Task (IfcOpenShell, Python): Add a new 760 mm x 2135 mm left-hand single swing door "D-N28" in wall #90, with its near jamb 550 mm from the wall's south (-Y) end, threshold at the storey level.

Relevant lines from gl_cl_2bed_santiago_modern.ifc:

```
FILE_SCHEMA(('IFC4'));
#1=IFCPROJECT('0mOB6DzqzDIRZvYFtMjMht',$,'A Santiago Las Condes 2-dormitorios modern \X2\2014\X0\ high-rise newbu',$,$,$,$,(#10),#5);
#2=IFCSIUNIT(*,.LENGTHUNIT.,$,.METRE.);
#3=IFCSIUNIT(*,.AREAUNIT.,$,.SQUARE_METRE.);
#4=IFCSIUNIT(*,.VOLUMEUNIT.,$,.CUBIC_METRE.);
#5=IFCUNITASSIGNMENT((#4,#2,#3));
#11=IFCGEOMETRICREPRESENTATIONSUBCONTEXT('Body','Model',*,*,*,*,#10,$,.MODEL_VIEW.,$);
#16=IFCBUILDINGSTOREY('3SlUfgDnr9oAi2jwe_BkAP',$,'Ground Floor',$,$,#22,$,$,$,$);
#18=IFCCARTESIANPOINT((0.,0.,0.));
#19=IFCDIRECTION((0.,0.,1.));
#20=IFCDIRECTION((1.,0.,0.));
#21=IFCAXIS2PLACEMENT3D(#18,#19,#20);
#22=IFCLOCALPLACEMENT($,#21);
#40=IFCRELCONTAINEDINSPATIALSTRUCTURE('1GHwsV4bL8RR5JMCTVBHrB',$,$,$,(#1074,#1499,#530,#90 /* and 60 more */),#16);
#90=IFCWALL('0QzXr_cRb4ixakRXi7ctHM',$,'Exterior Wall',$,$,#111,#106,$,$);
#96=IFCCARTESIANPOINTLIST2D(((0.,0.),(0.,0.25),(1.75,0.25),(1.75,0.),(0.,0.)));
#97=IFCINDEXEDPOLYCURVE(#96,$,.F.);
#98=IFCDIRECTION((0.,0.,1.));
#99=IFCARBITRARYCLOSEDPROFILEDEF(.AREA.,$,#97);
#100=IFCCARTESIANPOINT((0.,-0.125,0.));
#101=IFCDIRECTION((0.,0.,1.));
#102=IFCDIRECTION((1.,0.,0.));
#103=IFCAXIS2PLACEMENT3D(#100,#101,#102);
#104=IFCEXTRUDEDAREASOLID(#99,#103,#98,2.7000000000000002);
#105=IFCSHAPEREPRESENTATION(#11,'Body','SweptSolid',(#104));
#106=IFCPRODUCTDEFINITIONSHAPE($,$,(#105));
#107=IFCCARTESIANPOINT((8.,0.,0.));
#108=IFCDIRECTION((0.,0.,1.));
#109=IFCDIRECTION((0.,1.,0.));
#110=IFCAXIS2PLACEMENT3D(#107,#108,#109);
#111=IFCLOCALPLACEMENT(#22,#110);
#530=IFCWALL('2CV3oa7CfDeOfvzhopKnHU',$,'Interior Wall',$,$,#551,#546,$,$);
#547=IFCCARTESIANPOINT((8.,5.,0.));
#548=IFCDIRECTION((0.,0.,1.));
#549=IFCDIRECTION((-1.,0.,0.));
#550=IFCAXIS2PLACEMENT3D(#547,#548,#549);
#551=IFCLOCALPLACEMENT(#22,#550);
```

```python
import numpy as np
import ifcopenshell
import ifcopenshell.api.feature
import ifcopenshell.api.geometry
import ifcopenshell.api.root
import ifcopenshell.api.spatial
import ifcopenshell.geom
import ifcopenshell.util.element
import ifcopenshell.util.placement
import ifcopenshell.util.representation
import ifcopenshell.util.shape
import ifcopenshell.util.unit

model = ifcopenshell.open("gl_cl_2bed_santiago_modern.ifc")
unit_scale = ifcopenshell.util.unit.calculate_unit_scale(model)
settings = ifcopenshell.geom.settings()


def volume(element):
    """Net volume in cubic metres, openings subtracted."""
    shape = ifcopenshell.geom.create_shape(settings, element)
    return ifcopenshell.util.shape.get_volume(shape.geometry)


wall = model.by_guid("0QzXr_cRb4ixakRXi7ctHM")
storey = ifcopenshell.util.element.get_container(wall, ifc_class="IfcBuildingStorey")
context = ifcopenshell.util.representation.get_context(model, "Model", "Body", "MODEL_VIEW")
before = volume(wall)

width, height, from_end, sill = 0.76, 2.135, 0.55, 0.0  # metres

# The wall runs along its own X axis, and the end named is its -X end.
wall_shape = ifcopenshell.geom.create_shape(settings, wall)
x, y, z = ifcopenshell.util.shape.get_vertices(wall_shape.geometry).T
start = x.min() + from_end
face, thickness = float(y.min()), float(y.max() - y.min())
wall_matrix = ifcopenshell.util.placement.get_local_placement(wall.ObjectPlacement)
level = ifcopenshell.util.placement.get_local_placement(storey.ObjectPlacement)[2, 3]


def in_wall(x, y):
    """Placement at x, y metres in the wall's axes, at sill height."""
    matrix = wall_matrix.copy()
    matrix[:, 3] = wall_matrix @ np.array([x / unit_scale, y / unit_scale, 0.0, 1.0])
    matrix[2, 3] = level + sill / unit_scale
    return matrix


# Opening: a box that overshoots both wall faces by 50 mm.
opening = ifcopenshell.api.root.create_entity(model, ifc_class="IfcOpeningElement", predefined_type="OPENING")
box = ifcopenshell.api.geometry.add_wall_representation(
    model, context=context, length=width, height=height, thickness=thickness + 0.1
)
ifcopenshell.api.geometry.assign_representation(model, product=opening, representation=box)
ifcopenshell.api.geometry.edit_object_placement(model, product=opening, matrix=in_wall(start, face - 0.05), is_si=False)
ifcopenshell.api.feature.add_feature(model, feature=opening, element=wall)

door = ifcopenshell.api.root.create_entity(model, ifc_class="IfcDoor", name="D-N28", predefined_type="DOOR")
door.OverallWidth, door.OverallHeight = width / unit_scale, height / unit_scale
door.OperationType = "SINGLE_SWING_LEFT"
body = ifcopenshell.api.geometry.add_door_representation(
    model,
    context=context,
    overall_width=door.OverallWidth,
    overall_height=door.OverallHeight,
    operation_type="SINGLE_SWING_LEFT",
    lining_properties={"LiningDepth": thickness / unit_scale, "ThresholdDepth": thickness / unit_scale},
)
ifcopenshell.api.geometry.assign_representation(model, product=door, representation=body)
ifcopenshell.api.spatial.assign_container(model, products=[door], relating_structure=storey)
ifcopenshell.api.feature.add_filling(model, opening=opening, element=door)

# The lining spans the wall, so the door starts at the wall face.
ifcopenshell.api.geometry.edit_object_placement(model, product=door, matrix=in_wall(start, face), is_si=False)

after = volume(wall)

print(f"wall volume {before:.3f} -> {after:.3f} m3")

model.write("gl_cl_2bed_santiago_modern-out.ifc")
```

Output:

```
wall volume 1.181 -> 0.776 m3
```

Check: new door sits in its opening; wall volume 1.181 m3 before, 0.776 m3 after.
